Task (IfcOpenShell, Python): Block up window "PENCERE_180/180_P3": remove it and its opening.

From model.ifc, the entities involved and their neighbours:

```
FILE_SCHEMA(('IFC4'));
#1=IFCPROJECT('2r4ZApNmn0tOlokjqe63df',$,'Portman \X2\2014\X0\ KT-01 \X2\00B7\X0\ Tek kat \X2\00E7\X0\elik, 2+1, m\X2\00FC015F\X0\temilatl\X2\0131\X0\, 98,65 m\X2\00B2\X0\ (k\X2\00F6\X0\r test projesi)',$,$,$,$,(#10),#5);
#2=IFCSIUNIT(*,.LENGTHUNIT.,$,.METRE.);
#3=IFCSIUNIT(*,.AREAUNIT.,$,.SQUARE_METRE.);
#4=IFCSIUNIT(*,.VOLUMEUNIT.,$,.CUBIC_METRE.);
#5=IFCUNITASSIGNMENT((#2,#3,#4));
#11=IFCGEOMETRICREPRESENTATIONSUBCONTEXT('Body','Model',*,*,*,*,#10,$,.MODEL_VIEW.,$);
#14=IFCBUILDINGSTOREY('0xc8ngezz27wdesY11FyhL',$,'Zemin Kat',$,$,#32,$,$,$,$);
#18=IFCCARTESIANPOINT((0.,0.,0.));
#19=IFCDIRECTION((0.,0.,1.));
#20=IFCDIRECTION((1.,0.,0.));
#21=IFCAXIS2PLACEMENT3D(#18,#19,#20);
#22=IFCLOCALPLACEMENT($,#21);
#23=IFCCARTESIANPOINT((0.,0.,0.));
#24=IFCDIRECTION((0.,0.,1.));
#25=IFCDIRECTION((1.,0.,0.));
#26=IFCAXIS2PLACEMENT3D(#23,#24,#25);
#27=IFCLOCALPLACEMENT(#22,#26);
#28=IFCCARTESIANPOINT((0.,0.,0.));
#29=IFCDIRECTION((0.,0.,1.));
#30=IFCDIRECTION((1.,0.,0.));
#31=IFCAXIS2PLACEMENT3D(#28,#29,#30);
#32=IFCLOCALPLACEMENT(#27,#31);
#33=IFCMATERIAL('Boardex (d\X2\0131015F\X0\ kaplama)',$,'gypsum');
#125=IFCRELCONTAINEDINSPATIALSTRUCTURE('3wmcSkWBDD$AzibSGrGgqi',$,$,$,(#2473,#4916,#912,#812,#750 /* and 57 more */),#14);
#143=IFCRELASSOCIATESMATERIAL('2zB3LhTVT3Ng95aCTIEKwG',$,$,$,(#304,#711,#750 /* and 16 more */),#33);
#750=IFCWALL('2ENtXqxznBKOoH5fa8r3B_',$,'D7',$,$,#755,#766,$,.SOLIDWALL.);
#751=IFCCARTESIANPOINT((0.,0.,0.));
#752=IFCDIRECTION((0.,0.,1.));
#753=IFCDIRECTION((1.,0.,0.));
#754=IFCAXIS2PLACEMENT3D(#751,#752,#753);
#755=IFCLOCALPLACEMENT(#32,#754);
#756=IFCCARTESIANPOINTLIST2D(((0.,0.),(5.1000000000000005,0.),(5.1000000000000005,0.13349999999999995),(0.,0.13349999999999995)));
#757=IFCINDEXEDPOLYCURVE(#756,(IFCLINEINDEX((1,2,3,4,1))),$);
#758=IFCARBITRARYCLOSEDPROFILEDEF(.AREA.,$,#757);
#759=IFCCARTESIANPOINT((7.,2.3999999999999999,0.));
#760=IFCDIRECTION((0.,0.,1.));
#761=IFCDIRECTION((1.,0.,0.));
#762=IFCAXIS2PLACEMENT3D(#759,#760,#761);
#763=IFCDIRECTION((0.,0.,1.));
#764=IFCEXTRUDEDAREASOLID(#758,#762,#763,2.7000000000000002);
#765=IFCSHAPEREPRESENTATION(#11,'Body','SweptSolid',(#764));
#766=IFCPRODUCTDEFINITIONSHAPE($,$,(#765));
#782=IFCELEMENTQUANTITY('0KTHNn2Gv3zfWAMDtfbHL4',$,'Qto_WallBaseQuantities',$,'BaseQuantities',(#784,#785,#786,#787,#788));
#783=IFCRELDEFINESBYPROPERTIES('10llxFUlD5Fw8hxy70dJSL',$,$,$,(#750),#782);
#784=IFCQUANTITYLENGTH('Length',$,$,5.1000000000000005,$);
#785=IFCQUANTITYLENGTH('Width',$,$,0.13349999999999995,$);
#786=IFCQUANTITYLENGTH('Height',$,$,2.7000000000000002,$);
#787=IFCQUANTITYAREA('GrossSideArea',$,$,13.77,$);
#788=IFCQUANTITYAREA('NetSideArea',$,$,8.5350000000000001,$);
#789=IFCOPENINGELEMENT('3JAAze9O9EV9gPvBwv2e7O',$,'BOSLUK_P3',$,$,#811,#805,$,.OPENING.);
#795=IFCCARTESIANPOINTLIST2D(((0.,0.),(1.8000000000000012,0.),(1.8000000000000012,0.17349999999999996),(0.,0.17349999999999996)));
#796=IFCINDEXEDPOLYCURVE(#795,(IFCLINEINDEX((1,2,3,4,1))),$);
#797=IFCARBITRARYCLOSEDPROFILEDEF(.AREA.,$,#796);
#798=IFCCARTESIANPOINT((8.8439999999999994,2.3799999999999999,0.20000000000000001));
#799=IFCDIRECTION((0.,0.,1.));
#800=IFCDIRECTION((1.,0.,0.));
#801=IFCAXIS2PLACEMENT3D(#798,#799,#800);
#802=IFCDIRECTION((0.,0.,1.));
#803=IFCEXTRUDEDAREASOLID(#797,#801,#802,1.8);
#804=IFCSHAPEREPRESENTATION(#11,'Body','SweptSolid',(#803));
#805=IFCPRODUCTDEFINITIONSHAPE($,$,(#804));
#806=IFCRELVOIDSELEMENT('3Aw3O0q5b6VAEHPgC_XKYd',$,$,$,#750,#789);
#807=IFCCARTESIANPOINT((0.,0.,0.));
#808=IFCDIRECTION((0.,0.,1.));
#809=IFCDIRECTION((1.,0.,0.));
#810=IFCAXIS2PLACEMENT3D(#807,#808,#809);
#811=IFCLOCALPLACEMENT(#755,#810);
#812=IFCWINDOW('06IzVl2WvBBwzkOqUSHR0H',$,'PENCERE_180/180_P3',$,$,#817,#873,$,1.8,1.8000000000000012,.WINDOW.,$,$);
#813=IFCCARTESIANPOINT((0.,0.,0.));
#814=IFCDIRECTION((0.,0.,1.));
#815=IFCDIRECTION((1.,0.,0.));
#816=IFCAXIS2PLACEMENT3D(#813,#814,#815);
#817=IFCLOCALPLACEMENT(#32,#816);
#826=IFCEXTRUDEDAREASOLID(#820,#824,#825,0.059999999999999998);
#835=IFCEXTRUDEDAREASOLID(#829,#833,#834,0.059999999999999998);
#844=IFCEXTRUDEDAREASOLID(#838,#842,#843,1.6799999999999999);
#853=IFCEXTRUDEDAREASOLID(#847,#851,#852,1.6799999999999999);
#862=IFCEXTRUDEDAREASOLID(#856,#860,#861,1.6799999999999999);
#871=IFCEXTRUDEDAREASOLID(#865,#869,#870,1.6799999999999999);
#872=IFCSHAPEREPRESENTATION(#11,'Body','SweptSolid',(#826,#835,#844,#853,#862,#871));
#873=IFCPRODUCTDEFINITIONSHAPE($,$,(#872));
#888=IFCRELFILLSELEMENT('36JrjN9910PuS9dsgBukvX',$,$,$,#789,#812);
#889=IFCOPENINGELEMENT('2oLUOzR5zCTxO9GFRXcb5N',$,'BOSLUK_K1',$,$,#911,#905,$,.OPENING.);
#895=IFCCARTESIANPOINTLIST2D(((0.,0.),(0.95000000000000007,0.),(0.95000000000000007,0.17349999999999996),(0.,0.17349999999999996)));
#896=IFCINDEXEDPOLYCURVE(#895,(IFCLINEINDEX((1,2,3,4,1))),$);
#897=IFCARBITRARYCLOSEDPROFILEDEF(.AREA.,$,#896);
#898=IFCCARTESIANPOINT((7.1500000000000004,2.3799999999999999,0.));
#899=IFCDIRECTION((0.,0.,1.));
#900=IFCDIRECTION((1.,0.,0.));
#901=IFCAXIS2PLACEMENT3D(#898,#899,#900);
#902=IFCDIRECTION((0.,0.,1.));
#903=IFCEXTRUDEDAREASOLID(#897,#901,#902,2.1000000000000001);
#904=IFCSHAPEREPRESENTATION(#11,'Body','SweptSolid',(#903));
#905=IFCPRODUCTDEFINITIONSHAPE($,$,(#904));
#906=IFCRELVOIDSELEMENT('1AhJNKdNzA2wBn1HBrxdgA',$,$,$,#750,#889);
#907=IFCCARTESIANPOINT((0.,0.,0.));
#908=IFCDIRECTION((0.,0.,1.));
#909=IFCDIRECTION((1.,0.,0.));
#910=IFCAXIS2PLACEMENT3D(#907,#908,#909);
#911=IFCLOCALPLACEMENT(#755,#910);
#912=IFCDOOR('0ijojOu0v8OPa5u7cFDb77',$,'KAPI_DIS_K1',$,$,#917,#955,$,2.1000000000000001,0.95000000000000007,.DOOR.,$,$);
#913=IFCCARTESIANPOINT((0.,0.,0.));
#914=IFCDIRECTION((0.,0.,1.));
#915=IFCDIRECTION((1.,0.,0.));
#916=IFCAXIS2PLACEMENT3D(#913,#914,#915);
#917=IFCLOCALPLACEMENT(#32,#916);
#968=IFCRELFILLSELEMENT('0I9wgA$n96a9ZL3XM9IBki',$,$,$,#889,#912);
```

```python
import ifcopenshell
import ifcopenshell.api.feature
import ifcopenshell.api.pset
import ifcopenshell.api.root
import ifcopenshell.geom
import ifcopenshell.util.element
import ifcopenshell.util.shape
import ifcopenshell.util.unit

model = ifcopenshell.open("model.ifc")
area_scale = ifcopenshell.util.unit.calculate_unit_scale(model, "AREAUNIT")
settings = ifcopenshell.geom.settings()


def volume(element):
    """Net volume in cubic metres, openings subtracted."""
    shape = ifcopenshell.geom.create_shape(settings, element)
    return ifcopenshell.util.shape.get_volume(shape.geometry)


window = model.by_guid("06IzVl2WvBBwzkOqUSHR0H")
opening = window.FillsVoids[0].RelatingOpeningElement
wall = opening.VoidsElements[0].RelatingBuildingElement
before = volume(wall)

ifcopenshell.api.root.remove_product(model, product=window)
ifcopenshell.api.feature.remove_feature(model, feature=opening)

after = volume(wall)
thickness = 0.1335  # wall thickness in metres

# Update the wall's stored quantities.
qto = model.by_id(ifcopenshell.util.element.get_pset(wall, "Qto_WallBaseQuantities", should_inherit=False)["id"])
ifcopenshell.api.pset.edit_qto(model, qto=qto, properties={"NetSideArea": after / thickness / area_scale})

print(f"wall volume {before:.3f} -> {after:.3f} m3")

model.write("model_rev.ifc")
```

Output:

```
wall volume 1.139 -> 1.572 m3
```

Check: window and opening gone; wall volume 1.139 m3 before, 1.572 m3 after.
